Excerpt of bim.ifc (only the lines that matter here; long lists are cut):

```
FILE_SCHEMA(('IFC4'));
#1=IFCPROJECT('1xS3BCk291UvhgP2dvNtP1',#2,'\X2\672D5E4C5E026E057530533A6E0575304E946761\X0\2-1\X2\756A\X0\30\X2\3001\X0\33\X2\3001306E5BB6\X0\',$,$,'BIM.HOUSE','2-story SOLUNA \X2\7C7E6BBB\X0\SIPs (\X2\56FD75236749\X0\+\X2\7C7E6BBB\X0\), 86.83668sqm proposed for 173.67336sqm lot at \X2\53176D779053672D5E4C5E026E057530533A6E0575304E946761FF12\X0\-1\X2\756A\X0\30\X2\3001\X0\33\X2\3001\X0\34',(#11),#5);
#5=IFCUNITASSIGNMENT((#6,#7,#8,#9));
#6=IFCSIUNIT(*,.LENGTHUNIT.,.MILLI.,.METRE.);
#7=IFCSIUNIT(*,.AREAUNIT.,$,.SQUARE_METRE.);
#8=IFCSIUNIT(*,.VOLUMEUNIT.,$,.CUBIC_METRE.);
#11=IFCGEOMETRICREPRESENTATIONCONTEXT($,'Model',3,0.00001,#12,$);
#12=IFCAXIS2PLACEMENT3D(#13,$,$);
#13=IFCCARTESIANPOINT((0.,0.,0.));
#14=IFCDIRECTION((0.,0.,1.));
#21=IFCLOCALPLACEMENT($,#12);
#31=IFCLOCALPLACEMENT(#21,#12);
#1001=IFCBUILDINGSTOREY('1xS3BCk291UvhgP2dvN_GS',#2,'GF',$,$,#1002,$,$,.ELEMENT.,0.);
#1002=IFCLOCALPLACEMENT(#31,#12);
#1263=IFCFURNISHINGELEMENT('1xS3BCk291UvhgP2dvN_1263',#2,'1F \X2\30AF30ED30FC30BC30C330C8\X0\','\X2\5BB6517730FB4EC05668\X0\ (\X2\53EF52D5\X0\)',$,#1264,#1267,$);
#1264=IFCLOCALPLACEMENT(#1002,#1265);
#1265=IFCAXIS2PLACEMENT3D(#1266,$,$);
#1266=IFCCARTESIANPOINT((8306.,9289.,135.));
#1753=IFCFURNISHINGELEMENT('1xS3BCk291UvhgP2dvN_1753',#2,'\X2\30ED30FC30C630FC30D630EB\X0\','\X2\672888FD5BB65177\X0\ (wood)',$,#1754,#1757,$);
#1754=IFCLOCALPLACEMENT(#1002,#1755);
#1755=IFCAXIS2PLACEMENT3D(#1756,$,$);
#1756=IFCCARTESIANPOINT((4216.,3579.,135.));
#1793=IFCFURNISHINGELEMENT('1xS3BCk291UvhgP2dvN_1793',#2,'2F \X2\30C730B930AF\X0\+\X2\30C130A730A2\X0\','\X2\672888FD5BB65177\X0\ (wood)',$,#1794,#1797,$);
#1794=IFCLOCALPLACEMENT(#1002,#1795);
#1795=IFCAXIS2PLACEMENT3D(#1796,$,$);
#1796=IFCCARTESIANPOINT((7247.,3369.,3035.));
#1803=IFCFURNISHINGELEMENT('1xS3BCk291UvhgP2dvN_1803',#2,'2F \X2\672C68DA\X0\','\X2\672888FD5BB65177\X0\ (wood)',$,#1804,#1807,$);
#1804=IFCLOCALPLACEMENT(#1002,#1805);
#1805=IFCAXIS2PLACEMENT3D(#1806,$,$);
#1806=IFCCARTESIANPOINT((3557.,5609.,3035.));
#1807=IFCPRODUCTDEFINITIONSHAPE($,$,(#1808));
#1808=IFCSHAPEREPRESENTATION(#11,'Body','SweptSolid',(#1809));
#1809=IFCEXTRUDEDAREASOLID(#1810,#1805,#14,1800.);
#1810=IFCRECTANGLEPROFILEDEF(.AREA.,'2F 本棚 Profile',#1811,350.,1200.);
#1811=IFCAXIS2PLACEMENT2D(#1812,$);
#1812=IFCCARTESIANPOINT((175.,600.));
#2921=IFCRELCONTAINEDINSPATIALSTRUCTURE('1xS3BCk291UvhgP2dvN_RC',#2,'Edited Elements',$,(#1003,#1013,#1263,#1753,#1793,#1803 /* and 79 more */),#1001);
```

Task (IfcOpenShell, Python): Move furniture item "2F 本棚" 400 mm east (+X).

```python
import ifcopenshell
import ifcopenshell.api.geometry
import ifcopenshell.util.placement

model = ifcopenshell.open("bim.ifc")

item = model.by_guid("1xS3BCk291UvhgP2dvN_1803")
matrix = ifcopenshell.util.placement.get_local_placement(item.ObjectPlacement)
matrix[0, 3] += 400.0
ifcopenshell.api.geometry.edit_object_placement(model, product=item, matrix=matrix, is_si=False)

print(ifcopenshell.util.placement.get_local_placement(item.ObjectPlacement).round(3) + 0.0)

model.write("bim_edited.ifc")
```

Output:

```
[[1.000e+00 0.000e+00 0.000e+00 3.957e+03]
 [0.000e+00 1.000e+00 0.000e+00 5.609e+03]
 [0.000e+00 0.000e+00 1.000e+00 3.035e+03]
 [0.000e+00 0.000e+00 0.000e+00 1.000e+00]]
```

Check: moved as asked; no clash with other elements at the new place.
